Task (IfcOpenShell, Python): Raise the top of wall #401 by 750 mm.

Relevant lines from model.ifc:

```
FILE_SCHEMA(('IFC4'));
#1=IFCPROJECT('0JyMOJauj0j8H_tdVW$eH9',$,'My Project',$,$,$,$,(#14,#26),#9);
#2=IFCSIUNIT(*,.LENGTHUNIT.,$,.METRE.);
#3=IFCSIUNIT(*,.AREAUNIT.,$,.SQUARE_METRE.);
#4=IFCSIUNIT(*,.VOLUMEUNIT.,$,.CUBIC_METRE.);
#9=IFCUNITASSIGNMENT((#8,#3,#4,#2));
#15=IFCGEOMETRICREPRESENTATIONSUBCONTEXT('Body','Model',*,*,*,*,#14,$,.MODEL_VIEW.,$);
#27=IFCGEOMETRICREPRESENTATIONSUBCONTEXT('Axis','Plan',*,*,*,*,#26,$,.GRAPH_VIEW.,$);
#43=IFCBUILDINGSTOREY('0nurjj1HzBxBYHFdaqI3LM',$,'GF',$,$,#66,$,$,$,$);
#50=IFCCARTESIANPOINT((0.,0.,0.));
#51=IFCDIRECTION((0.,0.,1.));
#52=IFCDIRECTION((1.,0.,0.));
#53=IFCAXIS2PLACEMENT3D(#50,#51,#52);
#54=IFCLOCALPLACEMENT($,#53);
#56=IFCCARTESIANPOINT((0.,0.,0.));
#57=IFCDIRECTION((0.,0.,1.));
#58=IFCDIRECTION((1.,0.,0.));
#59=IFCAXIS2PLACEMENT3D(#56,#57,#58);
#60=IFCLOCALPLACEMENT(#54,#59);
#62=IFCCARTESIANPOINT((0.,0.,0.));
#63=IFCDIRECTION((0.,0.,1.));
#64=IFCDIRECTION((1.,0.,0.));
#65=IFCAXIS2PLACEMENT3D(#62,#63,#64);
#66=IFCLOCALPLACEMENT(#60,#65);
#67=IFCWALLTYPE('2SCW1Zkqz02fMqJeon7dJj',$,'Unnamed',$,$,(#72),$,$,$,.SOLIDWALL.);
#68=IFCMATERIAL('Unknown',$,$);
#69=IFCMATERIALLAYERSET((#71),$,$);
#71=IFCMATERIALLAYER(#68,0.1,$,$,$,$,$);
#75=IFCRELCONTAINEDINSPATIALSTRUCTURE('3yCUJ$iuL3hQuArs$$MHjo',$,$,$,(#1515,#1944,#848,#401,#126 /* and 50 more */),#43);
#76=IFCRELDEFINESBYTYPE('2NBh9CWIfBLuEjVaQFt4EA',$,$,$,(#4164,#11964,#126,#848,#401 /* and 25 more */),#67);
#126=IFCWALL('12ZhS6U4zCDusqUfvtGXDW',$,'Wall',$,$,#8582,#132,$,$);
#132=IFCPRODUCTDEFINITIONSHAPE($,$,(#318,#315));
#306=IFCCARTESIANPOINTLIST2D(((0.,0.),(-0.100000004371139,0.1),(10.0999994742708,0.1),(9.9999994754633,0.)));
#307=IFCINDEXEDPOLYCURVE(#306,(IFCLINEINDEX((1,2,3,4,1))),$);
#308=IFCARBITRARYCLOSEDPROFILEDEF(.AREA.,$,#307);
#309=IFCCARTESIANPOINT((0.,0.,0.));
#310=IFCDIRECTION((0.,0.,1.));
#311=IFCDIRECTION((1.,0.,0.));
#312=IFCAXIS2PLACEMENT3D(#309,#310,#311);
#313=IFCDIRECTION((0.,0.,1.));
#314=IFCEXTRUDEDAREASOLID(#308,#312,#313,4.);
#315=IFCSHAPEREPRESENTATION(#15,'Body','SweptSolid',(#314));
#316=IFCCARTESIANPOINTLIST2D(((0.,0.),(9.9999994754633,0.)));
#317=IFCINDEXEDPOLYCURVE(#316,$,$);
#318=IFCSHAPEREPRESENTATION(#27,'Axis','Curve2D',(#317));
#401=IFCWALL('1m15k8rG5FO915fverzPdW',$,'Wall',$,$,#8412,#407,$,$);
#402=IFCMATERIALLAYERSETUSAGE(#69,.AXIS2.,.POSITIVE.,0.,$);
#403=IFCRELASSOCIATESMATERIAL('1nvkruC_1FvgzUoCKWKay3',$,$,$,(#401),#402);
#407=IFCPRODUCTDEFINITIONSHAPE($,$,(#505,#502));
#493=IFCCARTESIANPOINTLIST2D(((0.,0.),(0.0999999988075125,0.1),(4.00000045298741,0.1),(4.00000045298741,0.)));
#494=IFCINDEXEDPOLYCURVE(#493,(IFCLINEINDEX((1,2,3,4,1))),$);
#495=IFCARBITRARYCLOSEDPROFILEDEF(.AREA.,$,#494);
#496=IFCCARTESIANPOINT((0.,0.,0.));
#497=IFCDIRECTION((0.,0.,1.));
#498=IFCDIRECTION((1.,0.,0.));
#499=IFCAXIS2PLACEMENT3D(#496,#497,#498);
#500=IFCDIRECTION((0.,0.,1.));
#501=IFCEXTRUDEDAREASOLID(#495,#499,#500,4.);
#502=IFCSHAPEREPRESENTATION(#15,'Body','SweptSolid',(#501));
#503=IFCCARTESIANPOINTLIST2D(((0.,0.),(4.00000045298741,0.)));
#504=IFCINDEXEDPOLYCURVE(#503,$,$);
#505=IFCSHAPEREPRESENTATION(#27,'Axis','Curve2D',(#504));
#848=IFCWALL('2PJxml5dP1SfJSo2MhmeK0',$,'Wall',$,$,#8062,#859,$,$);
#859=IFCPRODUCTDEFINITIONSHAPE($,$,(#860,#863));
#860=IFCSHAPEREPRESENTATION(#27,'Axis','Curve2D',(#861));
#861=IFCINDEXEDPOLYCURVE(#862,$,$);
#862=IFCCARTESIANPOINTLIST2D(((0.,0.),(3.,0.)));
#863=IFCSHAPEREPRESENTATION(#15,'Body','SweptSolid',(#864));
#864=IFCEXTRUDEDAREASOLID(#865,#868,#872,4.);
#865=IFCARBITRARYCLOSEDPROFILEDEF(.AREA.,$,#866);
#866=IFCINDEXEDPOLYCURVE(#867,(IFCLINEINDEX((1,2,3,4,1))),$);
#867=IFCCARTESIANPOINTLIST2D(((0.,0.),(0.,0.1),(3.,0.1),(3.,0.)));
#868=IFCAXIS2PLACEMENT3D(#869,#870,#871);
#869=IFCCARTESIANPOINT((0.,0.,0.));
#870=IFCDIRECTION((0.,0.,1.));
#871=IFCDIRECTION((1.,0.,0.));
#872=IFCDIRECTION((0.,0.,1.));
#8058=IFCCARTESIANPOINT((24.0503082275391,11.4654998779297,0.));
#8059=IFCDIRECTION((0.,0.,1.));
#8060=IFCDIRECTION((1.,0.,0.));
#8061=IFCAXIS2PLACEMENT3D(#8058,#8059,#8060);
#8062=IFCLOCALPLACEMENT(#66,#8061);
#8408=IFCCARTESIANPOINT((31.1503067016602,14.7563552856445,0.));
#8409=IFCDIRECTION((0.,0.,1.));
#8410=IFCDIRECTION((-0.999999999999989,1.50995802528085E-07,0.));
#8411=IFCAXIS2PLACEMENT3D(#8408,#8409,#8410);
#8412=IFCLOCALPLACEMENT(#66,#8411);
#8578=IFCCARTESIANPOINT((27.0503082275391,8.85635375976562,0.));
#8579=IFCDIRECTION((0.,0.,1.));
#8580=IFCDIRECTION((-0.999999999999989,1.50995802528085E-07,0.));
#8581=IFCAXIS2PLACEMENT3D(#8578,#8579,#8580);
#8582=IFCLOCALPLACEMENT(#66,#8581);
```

```python
import ifcopenshell
import ifcopenshell.geom
import ifcopenshell.util.representation
import ifcopenshell.util.shape

model = ifcopenshell.open("model.ifc")
settings = ifcopenshell.geom.settings()


def volume(element):
    """Net volume in cubic metres, openings subtracted."""
    shape = ifcopenshell.geom.create_shape(settings, element)
    return ifcopenshell.util.shape.get_volume(shape.geometry)


wall = model.by_guid("1m15k8rG5FO915fverzPdW")
before = volume(wall)

body = ifcopenshell.util.representation.get_representation(wall, "Model", "Body")
solid = body.Items[0]
old_height = solid.Depth
solid.Depth += 0.75
after = volume(wall)

print(f"height {old_height:g} -> {solid.Depth:g}, volume {before:.3f} -> {after:.3f} m3")

model.write("model_v2.ifc")
```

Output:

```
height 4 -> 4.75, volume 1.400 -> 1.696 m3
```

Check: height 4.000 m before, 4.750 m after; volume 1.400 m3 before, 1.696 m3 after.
